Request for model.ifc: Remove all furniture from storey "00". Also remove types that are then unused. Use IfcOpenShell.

First a look at what the model holds.

```python
import ifcopenshell
import ifcopenshell.util.element

model = ifcopenshell.open("model.ifc")
print(model.schema)
storey = next(s for s in model.by_type("IfcBuildingStorey") if s.Name == "00")
furniture = [e for e in ifcopenshell.util.element.get_decomposition(storey) if e.is_a("IfcFurnishingElement")]
seen = {}
for e in furniture:
    element_type = ifcopenshell.util.element.get_type(e)
    name = element_type.Name if element_type not in (None, e) else None
    seen[name] = seen.get(name, 0) + 1
for name, count in sorted(seen.items(), key=str):
    print(count, "x", name)
```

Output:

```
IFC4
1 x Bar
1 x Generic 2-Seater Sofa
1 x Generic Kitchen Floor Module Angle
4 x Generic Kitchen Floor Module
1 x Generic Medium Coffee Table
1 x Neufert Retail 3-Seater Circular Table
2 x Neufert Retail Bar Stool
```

```python
import ifcopenshell
import ifcopenshell.api.root
import ifcopenshell.util.element

model = ifcopenshell.open("model.ifc")

storey = next(s for s in model.by_type("IfcBuildingStorey") if s.Name == "00")
furniture = [e for e in ifcopenshell.util.element.get_decomposition(storey) if e.is_a("IfcFurnishingElement")]
types = {ifcopenshell.util.element.get_type(e) for e in furniture} - {None, *furniture}

for e in furniture:
    ifcopenshell.api.root.remove_product(model, product=e)
print(len(furniture), "removed")

unused = [t for t in types if not ifcopenshell.util.element.get_types(t)]
for t in unused:
    ifcopenshell.api.root.remove_product(model, product=t)
print(len(unused), "unused types removed")

model.write("model-out.ifc")
```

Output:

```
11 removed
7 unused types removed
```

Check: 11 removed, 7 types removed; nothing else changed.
